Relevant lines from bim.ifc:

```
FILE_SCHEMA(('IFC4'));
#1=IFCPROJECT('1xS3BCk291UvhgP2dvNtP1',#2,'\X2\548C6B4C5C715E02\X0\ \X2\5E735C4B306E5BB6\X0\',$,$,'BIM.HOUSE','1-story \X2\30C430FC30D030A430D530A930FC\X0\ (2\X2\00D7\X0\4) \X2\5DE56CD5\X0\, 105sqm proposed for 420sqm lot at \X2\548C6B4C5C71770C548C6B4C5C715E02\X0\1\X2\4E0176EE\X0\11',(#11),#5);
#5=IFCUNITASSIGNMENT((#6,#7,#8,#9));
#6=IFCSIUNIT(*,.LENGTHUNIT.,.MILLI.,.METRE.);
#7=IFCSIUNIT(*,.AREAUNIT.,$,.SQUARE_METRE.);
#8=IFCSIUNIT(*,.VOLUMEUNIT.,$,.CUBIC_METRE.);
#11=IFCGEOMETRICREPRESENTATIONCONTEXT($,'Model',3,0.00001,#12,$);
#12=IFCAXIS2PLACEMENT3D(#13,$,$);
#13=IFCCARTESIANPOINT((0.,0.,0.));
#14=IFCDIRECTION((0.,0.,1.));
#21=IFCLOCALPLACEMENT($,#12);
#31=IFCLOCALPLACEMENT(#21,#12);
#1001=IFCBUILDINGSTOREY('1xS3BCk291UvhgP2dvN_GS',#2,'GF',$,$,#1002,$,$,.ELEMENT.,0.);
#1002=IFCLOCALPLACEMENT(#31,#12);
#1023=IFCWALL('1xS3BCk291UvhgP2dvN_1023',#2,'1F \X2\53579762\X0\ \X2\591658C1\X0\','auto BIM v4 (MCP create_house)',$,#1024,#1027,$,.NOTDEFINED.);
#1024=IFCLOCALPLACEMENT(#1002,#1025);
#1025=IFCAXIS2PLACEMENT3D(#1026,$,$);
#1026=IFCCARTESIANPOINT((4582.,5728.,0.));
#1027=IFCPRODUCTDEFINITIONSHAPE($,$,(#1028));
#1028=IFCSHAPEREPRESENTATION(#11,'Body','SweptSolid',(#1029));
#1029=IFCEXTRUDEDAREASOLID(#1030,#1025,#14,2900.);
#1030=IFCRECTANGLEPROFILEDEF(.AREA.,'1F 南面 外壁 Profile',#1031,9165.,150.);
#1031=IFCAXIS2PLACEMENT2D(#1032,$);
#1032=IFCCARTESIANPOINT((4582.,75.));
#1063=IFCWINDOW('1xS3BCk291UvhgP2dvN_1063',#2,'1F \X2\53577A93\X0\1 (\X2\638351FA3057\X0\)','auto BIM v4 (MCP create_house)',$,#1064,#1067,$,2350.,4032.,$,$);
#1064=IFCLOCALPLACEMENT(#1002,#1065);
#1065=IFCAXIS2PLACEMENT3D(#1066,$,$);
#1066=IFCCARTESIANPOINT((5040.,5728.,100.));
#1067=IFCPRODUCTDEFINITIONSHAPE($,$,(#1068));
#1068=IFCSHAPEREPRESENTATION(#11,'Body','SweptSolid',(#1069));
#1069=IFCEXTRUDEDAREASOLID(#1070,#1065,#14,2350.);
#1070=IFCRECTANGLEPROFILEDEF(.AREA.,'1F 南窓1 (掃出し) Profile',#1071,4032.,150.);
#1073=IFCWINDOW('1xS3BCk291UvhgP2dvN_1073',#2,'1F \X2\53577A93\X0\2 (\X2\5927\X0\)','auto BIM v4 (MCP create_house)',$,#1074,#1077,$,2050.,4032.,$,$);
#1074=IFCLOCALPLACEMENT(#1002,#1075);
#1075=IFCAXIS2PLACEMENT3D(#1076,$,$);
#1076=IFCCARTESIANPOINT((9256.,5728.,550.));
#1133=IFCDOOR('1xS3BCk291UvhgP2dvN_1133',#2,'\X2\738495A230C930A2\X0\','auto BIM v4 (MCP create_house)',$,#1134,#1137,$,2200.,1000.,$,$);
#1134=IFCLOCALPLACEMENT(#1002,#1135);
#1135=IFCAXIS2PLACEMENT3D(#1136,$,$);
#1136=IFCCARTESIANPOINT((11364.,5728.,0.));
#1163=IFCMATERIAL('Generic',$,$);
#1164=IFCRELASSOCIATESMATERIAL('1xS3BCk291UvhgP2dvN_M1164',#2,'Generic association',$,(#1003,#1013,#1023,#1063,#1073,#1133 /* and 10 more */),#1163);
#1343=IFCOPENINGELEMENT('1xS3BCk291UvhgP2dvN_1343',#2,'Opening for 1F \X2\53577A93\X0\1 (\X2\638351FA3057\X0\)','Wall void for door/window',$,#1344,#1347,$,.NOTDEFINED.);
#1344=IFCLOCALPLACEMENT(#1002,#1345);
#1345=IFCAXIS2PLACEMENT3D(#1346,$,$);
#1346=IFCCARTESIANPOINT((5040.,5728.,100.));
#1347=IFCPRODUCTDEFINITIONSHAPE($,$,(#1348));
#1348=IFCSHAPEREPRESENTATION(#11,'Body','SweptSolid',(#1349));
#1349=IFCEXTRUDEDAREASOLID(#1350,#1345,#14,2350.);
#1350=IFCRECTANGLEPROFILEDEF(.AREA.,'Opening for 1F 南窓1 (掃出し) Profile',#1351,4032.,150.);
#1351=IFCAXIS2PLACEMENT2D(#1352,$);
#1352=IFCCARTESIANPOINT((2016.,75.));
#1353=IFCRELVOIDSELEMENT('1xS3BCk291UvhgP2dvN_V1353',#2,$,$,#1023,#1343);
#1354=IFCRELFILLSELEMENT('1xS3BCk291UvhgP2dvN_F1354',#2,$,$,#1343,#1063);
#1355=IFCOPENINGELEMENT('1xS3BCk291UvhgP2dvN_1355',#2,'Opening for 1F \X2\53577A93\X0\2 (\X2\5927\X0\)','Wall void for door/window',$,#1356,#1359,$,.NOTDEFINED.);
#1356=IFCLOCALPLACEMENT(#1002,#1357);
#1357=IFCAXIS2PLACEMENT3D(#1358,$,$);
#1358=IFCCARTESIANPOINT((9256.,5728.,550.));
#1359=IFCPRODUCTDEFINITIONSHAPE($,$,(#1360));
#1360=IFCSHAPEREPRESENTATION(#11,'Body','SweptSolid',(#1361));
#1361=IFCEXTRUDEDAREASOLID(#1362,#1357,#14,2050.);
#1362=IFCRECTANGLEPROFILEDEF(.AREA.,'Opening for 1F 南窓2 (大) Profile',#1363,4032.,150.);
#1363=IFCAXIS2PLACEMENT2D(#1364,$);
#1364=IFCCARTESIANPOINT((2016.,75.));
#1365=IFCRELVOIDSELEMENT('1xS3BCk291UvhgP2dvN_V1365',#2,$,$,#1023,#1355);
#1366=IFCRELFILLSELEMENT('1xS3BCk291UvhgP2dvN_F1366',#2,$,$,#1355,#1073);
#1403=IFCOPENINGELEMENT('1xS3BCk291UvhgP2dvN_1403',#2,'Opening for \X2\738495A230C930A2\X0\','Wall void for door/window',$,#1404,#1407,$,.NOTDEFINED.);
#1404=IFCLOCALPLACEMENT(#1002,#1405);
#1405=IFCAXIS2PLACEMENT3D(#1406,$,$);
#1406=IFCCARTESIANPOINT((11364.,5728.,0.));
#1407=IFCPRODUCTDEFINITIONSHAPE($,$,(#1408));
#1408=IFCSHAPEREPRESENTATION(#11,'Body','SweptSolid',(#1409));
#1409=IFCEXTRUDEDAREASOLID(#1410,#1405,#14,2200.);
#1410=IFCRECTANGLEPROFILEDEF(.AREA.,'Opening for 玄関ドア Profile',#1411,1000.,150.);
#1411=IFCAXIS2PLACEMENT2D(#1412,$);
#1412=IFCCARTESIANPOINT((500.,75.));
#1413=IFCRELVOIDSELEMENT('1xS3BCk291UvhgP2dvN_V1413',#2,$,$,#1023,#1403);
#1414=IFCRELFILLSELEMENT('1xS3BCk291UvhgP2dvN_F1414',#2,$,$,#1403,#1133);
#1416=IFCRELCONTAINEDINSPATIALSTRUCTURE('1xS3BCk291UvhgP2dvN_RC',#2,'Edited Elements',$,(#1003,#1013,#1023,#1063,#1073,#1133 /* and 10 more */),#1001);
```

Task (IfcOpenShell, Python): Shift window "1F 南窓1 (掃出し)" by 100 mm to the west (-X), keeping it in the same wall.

```python
import ifcopenshell
import ifcopenshell.api.geometry
import ifcopenshell.util.placement
import ifcopenshell.util.unit

model = ifcopenshell.open("bim.ifc")
unit_scale = ifcopenshell.util.unit.calculate_unit_scale(model)

window = model.by_id(1063)
opening = window.FillsVoids[0].RelatingOpeningElement
wall = opening.VoidsElements[0].RelatingBuildingElement

wall_matrix = ifcopenshell.util.placement.get_local_placement(wall.ObjectPlacement)
shift = wall_matrix[:3, 0] * -0.1 / unit_scale
before = ifcopenshell.util.placement.get_local_placement(window.ObjectPlacement)[:3, 3].copy()

# The window is not placed relative to its opening, so move both.
for product in (opening, window):
    matrix = ifcopenshell.util.placement.get_local_placement(product.ObjectPlacement)
    matrix[:3, 3] += shift
    ifcopenshell.api.geometry.edit_object_placement(model, product=product, matrix=matrix, is_si=False)

after = ifcopenshell.util.placement.get_local_placement(window.ObjectPlacement)[:3, 3]
print("window moved by", (after - before).round(3) + 0.0)

model.write("bim-out.ifc")
```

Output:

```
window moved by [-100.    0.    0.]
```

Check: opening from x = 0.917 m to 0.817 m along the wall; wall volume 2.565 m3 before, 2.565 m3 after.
